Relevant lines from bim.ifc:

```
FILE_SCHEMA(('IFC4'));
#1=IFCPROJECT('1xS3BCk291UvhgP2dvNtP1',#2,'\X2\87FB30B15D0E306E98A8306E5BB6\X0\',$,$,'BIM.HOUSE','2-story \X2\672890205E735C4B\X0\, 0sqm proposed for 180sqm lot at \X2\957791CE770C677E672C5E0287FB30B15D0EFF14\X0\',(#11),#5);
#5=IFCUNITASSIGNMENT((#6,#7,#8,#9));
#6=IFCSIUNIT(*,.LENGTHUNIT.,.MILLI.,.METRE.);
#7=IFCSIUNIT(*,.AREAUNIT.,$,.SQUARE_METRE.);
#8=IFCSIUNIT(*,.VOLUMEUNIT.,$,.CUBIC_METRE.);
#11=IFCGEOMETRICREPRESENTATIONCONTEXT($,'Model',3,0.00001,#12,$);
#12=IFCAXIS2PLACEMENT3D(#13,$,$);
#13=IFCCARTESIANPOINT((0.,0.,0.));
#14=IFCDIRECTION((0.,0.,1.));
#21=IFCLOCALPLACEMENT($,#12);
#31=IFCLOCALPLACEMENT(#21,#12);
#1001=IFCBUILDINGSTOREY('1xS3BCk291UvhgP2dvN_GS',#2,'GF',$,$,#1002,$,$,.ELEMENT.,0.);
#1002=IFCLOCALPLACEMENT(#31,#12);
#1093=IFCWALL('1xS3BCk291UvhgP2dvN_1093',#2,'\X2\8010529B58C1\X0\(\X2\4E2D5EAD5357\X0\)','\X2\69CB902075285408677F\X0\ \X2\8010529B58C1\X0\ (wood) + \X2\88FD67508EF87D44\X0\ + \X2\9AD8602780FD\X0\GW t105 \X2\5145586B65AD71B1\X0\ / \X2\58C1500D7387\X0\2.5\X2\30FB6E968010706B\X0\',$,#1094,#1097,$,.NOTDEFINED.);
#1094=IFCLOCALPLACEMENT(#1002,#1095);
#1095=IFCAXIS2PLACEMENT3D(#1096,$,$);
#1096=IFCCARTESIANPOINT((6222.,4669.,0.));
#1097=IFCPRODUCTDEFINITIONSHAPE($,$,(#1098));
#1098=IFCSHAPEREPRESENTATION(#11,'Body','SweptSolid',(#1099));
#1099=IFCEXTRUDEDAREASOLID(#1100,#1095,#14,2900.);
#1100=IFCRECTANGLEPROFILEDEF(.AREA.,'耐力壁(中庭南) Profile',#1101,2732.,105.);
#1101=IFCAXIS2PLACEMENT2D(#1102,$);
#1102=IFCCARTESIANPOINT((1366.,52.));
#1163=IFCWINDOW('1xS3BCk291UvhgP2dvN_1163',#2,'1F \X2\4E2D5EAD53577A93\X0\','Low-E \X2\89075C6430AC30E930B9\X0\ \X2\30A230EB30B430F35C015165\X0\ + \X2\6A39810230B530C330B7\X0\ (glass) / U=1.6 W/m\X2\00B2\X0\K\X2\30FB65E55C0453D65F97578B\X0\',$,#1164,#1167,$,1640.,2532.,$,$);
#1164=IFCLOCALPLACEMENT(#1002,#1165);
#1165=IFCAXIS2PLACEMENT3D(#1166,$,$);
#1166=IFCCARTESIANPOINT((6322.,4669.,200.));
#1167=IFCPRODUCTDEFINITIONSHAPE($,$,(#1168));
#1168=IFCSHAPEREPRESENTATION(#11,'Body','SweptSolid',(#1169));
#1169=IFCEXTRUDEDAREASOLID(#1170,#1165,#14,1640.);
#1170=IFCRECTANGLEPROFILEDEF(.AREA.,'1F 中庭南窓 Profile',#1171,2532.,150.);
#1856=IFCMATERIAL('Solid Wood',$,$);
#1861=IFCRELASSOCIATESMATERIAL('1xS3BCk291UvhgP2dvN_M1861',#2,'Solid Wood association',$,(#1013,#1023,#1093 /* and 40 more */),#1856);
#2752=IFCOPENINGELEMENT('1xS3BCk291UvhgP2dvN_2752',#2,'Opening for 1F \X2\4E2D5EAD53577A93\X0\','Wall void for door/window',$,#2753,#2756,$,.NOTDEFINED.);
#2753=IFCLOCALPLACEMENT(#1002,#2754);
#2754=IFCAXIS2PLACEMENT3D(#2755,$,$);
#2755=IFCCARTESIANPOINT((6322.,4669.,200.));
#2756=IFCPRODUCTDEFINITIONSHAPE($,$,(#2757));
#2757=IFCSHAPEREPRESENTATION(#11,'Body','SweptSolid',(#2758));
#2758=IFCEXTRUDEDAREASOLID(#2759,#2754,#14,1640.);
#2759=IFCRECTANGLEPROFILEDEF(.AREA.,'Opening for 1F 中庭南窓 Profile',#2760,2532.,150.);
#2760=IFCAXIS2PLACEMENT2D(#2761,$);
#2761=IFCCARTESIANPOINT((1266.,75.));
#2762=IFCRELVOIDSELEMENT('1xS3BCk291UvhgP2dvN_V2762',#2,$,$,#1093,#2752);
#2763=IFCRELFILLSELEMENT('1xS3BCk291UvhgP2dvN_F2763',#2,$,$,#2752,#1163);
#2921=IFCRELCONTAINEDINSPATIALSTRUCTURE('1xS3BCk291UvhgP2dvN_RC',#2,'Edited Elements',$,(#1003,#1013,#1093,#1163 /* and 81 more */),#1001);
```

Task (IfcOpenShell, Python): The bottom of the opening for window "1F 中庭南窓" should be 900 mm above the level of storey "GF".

```python
import numpy as np
import ifcopenshell
import ifcopenshell.api.geometry
import ifcopenshell.geom
import ifcopenshell.util.element
import ifcopenshell.util.placement
import ifcopenshell.util.shape
import ifcopenshell.util.unit

model = ifcopenshell.open("bim.ifc")
unit_scale = ifcopenshell.util.unit.calculate_unit_scale(model)

window = model.by_guid("1xS3BCk291UvhgP2dvN_1163")
opening = window.FillsVoids[0].RelatingOpeningElement
storey = ifcopenshell.util.element.get_container(window, ifc_class="IfcBuildingStorey")
level = ifcopenshell.util.placement.get_local_placement(storey.ObjectPlacement)[2, 3]

# The opening's origin need not be at the sill, so measure its lowest point.
shape = ifcopenshell.geom.create_shape(ifcopenshell.geom.settings(), opening)
bottom = ifcopenshell.util.shape.get_shape_bottom_elevation(shape, shape.geometry) / unit_scale
dz = level + 900.0 - bottom

shift = np.array([0.0, 0.0, dz])
# The window is not placed relative to its opening, so move both.
for product in (opening, window):
    matrix = ifcopenshell.util.placement.get_local_placement(product.ObjectPlacement)
    matrix[:3, 3] += shift
    ifcopenshell.api.geometry.edit_object_placement(model, product=product, matrix=matrix, is_si=False)

print(f"moved by {dz * unit_scale:+.3f} m")

model.write("bim_rev.ifc")
```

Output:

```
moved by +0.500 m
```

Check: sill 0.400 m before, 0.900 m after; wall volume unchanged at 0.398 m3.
